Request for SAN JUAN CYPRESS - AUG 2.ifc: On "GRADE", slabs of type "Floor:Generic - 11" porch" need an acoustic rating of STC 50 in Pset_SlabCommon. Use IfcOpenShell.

First a look at what the model holds.

```python
import ifcopenshell
import ifcopenshell.util.element

model = ifcopenshell.open("SAN JUAN CYPRESS - AUG 2.ifc")
print(model.schema)
storey = next(s for s in model.by_type("IfcBuildingStorey") if s.Name == "GRADE")
slabs = [e for e in ifcopenshell.util.element.get_decomposition(storey) if e.is_a("IfcSlab")]
seen = {}
for e in slabs:
    element_type = ifcopenshell.util.element.get_type(e)
    key = (element_type.Name if element_type != e and element_type else None, ifcopenshell.util.element.get_pset(e, "Pset_SlabCommon", "AcousticRating"))
    seen[key] = seen.get(key, 0) + 1
for (name, value), count in sorted(seen.items(), key=str):
    print(count, "x", name, "|", value)
```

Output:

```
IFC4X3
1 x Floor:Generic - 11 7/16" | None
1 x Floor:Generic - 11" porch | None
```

```python
import ifcopenshell
import ifcopenshell.api.pset
import ifcopenshell.util.element

model = ifcopenshell.open("SAN JUAN CYPRESS - AUG 2.ifc")

storey = next(s for s in model.by_type("IfcBuildingStorey") if s.Name == "GRADE")
slabs = [e for e in ifcopenshell.util.element.get_decomposition(storey) if e.is_a("IfcSlab")]

count = 0
for e in slabs:
    element_type = ifcopenshell.util.element.get_type(e)
    if element_type in (None, e) or element_type.Name != 'Floor:Generic - 11" porch':
        continue
    # add_pset returns the element's existing set when there is one.
    pset = ifcopenshell.api.pset.add_pset(model, product=e, name="Pset_SlabCommon")
    ifcopenshell.api.pset.edit_pset(model, pset=pset, properties={"AcousticRating": "STC 50"})
    count += 1

print(count, "slabs updated")

model.write("SAN JUAN CYPRESS - AUG 2_edited.ifc")
```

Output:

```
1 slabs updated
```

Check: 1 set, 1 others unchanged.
